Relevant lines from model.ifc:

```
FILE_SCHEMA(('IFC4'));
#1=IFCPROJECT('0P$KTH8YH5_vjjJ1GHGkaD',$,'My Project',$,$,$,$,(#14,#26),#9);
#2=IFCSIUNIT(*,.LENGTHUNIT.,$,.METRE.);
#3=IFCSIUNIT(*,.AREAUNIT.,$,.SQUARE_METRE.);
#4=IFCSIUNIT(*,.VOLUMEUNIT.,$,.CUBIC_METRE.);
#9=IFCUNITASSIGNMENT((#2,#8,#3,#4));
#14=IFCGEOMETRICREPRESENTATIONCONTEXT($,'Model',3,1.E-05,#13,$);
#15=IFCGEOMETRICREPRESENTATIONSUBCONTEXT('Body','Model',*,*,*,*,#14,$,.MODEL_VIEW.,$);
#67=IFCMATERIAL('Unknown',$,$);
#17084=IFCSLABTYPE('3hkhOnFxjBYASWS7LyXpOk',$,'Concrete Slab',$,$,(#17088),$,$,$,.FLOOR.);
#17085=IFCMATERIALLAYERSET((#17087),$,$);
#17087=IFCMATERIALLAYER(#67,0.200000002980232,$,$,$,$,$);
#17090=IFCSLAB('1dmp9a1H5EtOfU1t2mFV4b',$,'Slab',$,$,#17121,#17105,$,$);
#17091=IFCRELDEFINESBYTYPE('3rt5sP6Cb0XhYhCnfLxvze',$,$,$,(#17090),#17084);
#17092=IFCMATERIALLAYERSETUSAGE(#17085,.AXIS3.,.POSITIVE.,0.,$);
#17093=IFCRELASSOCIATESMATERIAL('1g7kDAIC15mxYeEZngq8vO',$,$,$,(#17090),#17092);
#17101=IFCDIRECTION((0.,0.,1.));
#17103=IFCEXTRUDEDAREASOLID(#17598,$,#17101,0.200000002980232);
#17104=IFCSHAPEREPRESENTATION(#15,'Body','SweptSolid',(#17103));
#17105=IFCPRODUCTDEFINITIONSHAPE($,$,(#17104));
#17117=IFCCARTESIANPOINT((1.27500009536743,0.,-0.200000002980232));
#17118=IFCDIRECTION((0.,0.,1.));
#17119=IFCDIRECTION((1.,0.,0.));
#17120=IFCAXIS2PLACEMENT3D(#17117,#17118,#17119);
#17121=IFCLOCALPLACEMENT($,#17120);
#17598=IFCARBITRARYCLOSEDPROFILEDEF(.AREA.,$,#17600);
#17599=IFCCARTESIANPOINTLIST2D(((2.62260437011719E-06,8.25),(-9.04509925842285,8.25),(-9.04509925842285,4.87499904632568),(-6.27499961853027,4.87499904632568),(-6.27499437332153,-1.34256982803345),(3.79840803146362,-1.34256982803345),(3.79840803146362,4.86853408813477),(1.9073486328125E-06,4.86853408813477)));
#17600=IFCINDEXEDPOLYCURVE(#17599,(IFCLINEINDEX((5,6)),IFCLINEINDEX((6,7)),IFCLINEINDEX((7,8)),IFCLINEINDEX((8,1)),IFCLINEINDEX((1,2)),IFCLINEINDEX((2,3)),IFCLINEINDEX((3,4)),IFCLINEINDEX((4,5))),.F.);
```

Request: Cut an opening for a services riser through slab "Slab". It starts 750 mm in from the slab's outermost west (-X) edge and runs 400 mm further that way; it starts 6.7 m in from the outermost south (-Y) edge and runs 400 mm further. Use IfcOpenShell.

```python
import numpy as np
import ifcopenshell
import ifcopenshell.api.feature
import ifcopenshell.api.geometry
import ifcopenshell.api.root
import ifcopenshell.geom
import ifcopenshell.util.placement
import ifcopenshell.util.representation
import ifcopenshell.util.shape
import ifcopenshell.util.unit

model = ifcopenshell.open("model.ifc")
unit_scale = ifcopenshell.util.unit.calculate_unit_scale(model)
settings = ifcopenshell.geom.settings()


def volume(element):
    """Net volume in cubic metres, openings subtracted."""
    shape = ifcopenshell.geom.create_shape(settings, element)
    return ifcopenshell.util.shape.get_volume(shape.geometry)


slab = model.by_id(17090)
before = volume(slab)

# Extent in the slab's own axes, in metres. The edges named are its -X and -Y sides.
slab_shape = ifcopenshell.geom.create_shape(settings, slab)
vertices = ifcopenshell.util.shape.get_vertices(slab_shape.geometry)
x_min, y_min, bottom = vertices.min(axis=0)
top = vertices[:, 2].max()

opening = ifcopenshell.api.root.create_entity(model, ifc_class="IfcOpeningElement", name="Services riser opening", predefined_type="OPENING")
context = ifcopenshell.util.representation.get_context(model, "Model", "Body", "MODEL_VIEW")
width, depth = 0.4, 0.4
outline = [(0.0, 0.0), (width, 0.0), (width, depth), (0.0, depth), (0.0, 0.0)]
# Overshoot both faces by 50 mm so the cut is clean.
shape = ifcopenshell.api.geometry.add_slab_representation(
    model, context=context, depth=top - bottom + 0.1, polyline=outline
)
ifcopenshell.api.geometry.assign_representation(model, product=opening, representation=shape)

matrix = ifcopenshell.util.placement.get_local_placement(slab.ObjectPlacement)
matrix[:, 3] = matrix @ np.append(np.array([x_min + 0.75, y_min + 6.7, bottom - 0.05]) / unit_scale, 1.0)
ifcopenshell.api.geometry.edit_object_placement(model, product=opening, matrix=matrix, is_si=False)
ifcopenshell.api.feature.add_feature(model, feature=opening, element=slab)

after = volume(slab)

print(f"slab volume {before:.3f} -> {after:.3f} m3")

model.write("model_v2.ifc")
```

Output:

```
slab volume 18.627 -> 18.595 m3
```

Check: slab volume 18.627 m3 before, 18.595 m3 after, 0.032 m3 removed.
